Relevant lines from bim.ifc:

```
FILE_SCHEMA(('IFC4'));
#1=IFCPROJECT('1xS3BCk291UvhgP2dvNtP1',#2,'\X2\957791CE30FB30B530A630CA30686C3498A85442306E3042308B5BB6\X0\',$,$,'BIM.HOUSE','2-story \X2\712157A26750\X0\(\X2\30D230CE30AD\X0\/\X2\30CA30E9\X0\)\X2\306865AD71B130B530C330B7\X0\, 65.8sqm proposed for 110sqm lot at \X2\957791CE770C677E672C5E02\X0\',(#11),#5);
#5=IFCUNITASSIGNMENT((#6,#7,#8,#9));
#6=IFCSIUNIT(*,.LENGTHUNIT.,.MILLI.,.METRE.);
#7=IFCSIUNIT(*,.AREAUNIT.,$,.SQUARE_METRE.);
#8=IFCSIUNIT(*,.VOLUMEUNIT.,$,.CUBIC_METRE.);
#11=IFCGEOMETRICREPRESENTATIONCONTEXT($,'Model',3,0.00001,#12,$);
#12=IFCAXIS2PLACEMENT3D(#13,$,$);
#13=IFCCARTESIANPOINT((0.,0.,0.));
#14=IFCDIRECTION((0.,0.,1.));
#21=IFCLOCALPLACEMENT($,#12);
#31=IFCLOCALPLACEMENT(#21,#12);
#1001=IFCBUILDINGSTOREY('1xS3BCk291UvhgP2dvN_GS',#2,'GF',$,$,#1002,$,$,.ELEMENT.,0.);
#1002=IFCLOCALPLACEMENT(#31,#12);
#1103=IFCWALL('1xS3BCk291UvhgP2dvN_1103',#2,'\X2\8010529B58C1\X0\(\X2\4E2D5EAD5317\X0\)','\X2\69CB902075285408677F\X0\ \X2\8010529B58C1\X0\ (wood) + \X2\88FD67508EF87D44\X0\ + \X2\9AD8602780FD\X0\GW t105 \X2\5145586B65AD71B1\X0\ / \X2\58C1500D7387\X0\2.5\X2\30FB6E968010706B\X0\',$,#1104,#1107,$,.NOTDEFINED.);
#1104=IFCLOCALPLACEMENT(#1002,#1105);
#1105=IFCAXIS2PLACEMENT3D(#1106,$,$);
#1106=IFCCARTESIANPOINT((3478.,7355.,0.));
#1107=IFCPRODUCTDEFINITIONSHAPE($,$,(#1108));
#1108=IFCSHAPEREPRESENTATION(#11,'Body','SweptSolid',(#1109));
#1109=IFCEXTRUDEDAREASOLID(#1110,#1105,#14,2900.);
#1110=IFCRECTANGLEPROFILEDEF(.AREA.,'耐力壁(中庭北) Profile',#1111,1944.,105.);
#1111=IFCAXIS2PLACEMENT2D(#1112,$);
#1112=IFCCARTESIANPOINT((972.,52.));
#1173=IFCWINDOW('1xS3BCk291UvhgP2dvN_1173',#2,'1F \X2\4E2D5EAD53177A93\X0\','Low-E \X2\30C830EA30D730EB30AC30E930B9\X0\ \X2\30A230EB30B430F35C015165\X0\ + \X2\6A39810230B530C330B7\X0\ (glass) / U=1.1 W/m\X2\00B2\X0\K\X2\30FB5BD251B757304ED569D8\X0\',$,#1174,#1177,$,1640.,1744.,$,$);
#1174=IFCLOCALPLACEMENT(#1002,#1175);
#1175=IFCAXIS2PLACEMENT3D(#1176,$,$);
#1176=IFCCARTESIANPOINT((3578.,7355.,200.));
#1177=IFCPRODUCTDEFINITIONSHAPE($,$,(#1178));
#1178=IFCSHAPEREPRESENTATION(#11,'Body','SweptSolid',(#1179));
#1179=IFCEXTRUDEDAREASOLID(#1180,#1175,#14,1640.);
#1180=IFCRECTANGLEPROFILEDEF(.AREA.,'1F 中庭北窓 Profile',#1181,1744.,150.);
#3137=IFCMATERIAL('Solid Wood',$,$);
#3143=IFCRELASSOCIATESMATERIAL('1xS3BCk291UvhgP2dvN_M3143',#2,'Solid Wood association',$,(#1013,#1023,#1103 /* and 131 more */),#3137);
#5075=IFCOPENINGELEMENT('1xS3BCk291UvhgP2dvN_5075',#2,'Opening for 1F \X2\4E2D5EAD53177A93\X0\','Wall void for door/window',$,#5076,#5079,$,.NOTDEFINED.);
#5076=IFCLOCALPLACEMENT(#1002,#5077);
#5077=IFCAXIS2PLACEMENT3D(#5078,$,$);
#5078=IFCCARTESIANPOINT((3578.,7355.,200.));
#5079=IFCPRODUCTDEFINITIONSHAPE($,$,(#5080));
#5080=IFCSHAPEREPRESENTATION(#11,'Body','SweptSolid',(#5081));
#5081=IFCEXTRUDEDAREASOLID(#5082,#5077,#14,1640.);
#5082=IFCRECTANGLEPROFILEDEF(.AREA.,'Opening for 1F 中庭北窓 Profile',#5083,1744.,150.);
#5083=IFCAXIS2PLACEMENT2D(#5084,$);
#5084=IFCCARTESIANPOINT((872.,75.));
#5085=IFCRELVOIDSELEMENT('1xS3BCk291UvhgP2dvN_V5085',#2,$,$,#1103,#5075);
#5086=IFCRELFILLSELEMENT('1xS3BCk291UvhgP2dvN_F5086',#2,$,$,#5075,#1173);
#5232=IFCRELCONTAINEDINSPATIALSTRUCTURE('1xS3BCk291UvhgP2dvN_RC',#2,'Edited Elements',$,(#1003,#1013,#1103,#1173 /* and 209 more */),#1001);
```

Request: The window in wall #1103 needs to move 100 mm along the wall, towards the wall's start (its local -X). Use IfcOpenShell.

```python
import ifcopenshell
import ifcopenshell.api.geometry
import ifcopenshell.util.placement

model = ifcopenshell.open("bim.ifc")

window = model.by_id(1173)
opening = window.FillsVoids[0].RelatingOpeningElement
wall = opening.VoidsElements[0].RelatingBuildingElement

wall_matrix = ifcopenshell.util.placement.get_local_placement(wall.ObjectPlacement)
shift = wall_matrix[:3, 0] * -100.0
before = ifcopenshell.util.placement.get_local_placement(window.ObjectPlacement)[:3, 3].copy()

# The window is not placed relative to its opening, so move both.
for product in (opening, window):
    matrix = ifcopenshell.util.placement.get_local_placement(product.ObjectPlacement)
    matrix[:3, 3] += shift
    ifcopenshell.api.geometry.edit_object_placement(model, product=product, matrix=matrix, is_si=False)

after = ifcopenshell.util.placement.get_local_placement(window.ObjectPlacement)[:3, 3]
print("window moved by", (after - before).round(3) + 0.0)

model.write("bim_edited.ifc")
```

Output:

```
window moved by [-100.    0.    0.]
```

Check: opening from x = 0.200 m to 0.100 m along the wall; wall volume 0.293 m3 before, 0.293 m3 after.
